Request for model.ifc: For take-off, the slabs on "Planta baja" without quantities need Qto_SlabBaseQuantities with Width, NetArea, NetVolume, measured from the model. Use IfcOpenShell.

First a look at what the model holds.

```python
import ifcopenshell
import ifcopenshell.util.element
import ifcopenshell.util.unit

model = ifcopenshell.open("model.ifc")
print(model.schema)
for unit_type in ("LENGTHUNIT", "AREAUNIT", "VOLUMEUNIT"):
    print(unit_type, ifcopenshell.util.unit.calculate_unit_scale(model, unit_type))
storey = next(s for s in model.by_type("IfcBuildingStorey") if s.Name == "Planta baja")
slabs = [e for e in ifcopenshell.util.element.get_decomposition(storey) if e.is_a("IfcSlab")]
for e in sorted(slabs, key=lambda e: e.id()):
    print(e.id(), e.is_a(), e.Name, list(ifcopenshell.util.element.get_psets(e, qtos_only=True)), sep=" | ")
```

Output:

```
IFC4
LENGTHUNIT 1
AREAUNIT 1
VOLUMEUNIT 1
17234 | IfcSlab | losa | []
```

```python
import ifcopenshell
import ifcopenshell.api.pset
import ifcopenshell.geom
import ifcopenshell.util.element
import ifcopenshell.util.shape
import ifcopenshell.util.unit

model = ifcopenshell.open("model.ifc")
unit_scale = ifcopenshell.util.unit.calculate_unit_scale(model)
area_scale = ifcopenshell.util.unit.calculate_unit_scale(model, "AREAUNIT")
volume_scale = ifcopenshell.util.unit.calculate_unit_scale(model, "VOLUMEUNIT")
settings = ifcopenshell.geom.settings()

storey = next(s for s in model.by_type("IfcBuildingStorey") if s.Name == "Planta baja")
slabs = [e for e in ifcopenshell.util.element.get_decomposition(storey) if e.is_a("IfcSlab")]

for e in sorted(slabs, key=lambda e: e.id()):
    if ifcopenshell.util.element.get_psets(e, qtos_only=True, should_inherit=False):
        continue
    # Geometry comes back in metres, in the element's own axes.
    shape = ifcopenshell.geom.create_shape(settings, e)
    values = {
        "Width": ifcopenshell.util.shape.get_z(shape.geometry) / unit_scale,
        "NetArea": ifcopenshell.util.shape.get_footprint_area(shape.geometry) / area_scale,
        "NetVolume": ifcopenshell.util.shape.get_volume(shape.geometry) / volume_scale,
    }
    qto = ifcopenshell.api.pset.add_qto(model, product=e, name="Qto_SlabBaseQuantities")
    ifcopenshell.api.pset.edit_qto(model, qto=qto, properties=values)
    print(e.id(), {k: round(v, 3) for k, v in values.items()})

model.write("model_edited.ifc")
```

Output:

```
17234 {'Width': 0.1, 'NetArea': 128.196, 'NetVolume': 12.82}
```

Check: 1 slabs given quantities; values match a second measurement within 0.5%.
